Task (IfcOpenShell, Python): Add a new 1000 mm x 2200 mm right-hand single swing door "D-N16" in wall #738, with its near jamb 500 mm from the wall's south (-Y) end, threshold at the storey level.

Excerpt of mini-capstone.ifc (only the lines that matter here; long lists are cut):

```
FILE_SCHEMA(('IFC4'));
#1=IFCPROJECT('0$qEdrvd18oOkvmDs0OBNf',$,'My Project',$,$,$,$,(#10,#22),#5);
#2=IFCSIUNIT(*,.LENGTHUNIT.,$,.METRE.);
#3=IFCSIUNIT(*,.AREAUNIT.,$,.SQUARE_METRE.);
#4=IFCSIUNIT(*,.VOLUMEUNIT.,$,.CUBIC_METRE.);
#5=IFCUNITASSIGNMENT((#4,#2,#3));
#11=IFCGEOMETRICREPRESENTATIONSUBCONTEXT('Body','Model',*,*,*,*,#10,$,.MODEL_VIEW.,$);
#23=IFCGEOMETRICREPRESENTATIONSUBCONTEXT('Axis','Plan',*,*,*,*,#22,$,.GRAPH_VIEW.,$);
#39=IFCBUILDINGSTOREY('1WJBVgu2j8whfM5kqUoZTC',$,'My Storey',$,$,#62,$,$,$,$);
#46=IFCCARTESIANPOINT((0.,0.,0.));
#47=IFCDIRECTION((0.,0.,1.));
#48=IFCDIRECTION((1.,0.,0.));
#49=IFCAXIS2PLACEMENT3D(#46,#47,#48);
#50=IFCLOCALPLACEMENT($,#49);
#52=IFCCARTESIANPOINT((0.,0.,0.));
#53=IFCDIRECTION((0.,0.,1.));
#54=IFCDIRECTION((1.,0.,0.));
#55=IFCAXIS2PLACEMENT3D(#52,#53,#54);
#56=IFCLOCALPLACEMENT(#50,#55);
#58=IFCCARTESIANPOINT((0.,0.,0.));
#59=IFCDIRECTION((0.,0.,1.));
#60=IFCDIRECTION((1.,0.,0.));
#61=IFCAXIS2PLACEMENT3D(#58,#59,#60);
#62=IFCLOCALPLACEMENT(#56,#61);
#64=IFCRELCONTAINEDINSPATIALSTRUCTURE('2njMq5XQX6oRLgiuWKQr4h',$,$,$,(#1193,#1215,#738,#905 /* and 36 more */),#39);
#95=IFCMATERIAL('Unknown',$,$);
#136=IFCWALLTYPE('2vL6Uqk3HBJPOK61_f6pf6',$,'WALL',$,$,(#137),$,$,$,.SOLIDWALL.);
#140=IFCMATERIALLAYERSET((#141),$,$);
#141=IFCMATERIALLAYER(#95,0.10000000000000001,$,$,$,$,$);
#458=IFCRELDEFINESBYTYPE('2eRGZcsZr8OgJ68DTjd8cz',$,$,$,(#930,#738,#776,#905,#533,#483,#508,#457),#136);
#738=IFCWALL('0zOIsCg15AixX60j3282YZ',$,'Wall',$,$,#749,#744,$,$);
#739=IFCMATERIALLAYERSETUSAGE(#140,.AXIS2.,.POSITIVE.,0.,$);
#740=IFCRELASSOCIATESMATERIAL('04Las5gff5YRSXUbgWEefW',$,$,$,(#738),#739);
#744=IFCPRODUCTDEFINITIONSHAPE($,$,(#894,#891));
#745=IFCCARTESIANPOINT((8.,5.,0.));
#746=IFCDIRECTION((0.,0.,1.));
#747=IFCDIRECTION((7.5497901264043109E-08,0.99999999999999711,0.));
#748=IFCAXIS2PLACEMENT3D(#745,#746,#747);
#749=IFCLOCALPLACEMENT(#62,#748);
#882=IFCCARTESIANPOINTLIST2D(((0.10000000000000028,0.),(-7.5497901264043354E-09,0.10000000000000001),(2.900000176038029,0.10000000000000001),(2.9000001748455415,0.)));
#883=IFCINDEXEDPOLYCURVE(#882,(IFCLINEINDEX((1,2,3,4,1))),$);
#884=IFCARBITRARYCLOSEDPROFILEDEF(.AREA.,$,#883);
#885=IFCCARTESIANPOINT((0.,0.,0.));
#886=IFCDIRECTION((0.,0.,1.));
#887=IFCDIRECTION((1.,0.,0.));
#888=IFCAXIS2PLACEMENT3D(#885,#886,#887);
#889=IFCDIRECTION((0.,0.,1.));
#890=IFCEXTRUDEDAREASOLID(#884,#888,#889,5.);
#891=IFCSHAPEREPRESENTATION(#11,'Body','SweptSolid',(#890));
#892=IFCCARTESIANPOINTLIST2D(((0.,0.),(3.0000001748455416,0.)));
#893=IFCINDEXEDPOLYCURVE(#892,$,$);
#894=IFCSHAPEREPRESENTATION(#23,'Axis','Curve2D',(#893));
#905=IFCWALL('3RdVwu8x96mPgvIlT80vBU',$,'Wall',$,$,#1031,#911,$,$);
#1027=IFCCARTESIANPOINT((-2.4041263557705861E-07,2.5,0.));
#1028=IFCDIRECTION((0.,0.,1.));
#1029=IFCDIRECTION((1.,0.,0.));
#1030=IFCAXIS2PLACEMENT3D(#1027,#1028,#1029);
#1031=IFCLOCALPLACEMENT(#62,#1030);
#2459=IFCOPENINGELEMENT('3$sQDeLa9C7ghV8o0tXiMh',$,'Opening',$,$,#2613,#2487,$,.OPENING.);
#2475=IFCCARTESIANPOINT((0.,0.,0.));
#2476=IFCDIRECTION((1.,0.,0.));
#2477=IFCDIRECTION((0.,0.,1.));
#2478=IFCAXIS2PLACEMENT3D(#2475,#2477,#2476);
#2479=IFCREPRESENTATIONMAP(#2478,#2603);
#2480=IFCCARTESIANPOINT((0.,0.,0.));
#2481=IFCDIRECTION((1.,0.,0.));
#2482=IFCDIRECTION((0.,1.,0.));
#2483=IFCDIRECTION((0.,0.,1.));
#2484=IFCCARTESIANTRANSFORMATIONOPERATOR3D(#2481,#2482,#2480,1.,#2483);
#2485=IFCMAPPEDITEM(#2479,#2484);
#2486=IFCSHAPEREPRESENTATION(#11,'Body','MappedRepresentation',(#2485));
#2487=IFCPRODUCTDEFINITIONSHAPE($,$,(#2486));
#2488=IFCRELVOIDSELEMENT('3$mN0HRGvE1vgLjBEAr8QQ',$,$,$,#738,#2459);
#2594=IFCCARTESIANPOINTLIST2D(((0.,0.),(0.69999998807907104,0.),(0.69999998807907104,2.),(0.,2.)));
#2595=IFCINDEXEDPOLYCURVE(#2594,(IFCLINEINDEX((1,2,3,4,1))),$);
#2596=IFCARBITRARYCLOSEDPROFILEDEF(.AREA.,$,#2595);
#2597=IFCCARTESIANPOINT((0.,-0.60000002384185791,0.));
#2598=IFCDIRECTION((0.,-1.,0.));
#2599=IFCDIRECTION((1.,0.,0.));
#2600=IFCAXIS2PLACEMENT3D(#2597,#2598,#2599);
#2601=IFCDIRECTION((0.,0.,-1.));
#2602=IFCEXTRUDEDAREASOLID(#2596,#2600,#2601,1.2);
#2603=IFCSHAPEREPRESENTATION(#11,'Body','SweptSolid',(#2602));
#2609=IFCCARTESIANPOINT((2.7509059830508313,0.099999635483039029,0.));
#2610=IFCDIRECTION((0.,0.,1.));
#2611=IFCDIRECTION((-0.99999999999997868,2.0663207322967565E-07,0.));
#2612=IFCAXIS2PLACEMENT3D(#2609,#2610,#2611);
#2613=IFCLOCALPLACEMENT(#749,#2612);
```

```python
import numpy as np
import ifcopenshell
import ifcopenshell.api.feature
import ifcopenshell.api.geometry
import ifcopenshell.api.root
import ifcopenshell.api.spatial
import ifcopenshell.geom
import ifcopenshell.util.element
import ifcopenshell.util.placement
import ifcopenshell.util.representation
import ifcopenshell.util.shape
import ifcopenshell.util.unit

model = ifcopenshell.open("mini-capstone.ifc")
unit_scale = ifcopenshell.util.unit.calculate_unit_scale(model)
settings = ifcopenshell.geom.settings()


def volume(element):
    """Net volume in cubic metres, openings subtracted."""
    shape = ifcopenshell.geom.create_shape(settings, element)
    return ifcopenshell.util.shape.get_volume(shape.geometry)


wall = model.by_guid("0zOIsCg15AixX60j3282YZ")
storey = ifcopenshell.util.element.get_container(wall, ifc_class="IfcBuildingStorey")
context = ifcopenshell.util.representation.get_context(model, "Model", "Body", "MODEL_VIEW")
before = volume(wall)

width, height, from_end, sill = 1, 2.2, 0.5, 0.0  # metres

# The wall runs along its own X axis, and the end named is its -X end.
wall_shape = ifcopenshell.geom.create_shape(settings, wall)
x, y, z = ifcopenshell.util.shape.get_vertices(wall_shape.geometry).T
start = x.min() + from_end
face, thickness = float(y.min()), float(y.max() - y.min())
wall_matrix = ifcopenshell.util.placement.get_local_placement(wall.ObjectPlacement)
level = ifcopenshell.util.placement.get_local_placement(storey.ObjectPlacement)[2, 3]


def in_wall(x, y):
    """Placement at x, y metres in the wall's axes, at sill height."""
    matrix = wall_matrix.copy()
    matrix[:, 3] = wall_matrix @ np.array([x / unit_scale, y / unit_scale, 0.0, 1.0])
    matrix[2, 3] = level + sill / unit_scale
    return matrix


# Opening: a box that overshoots both wall faces by 50 mm.
opening = ifcopenshell.api.root.create_entity(model, ifc_class="IfcOpeningElement", predefined_type="OPENING")
box = ifcopenshell.api.geometry.add_wall_representation(
    model, context=context, length=width, height=height, thickness=thickness + 0.1
)
ifcopenshell.api.geometry.assign_representation(model, product=opening, representation=box)
ifcopenshell.api.geometry.edit_object_placement(model, product=opening, matrix=in_wall(start, face - 0.05), is_si=False)
ifcopenshell.api.feature.add_feature(model, feature=opening, element=wall)

door = ifcopenshell.api.root.create_entity(model, ifc_class="IfcDoor", name="D-N16", predefined_type="DOOR")
door.OverallWidth, door.OverallHeight = width / unit_scale, height / unit_scale
door.OperationType = "SINGLE_SWING_RIGHT"
body = ifcopenshell.api.geometry.add_door_representation(
    model,
    context=context,
    overall_width=door.OverallWidth,
    overall_height=door.OverallHeight,
    operation_type="SINGLE_SWING_RIGHT",
    lining_properties={"LiningDepth": thickness / unit_scale, "ThresholdDepth": thickness / unit_scale},
)
ifcopenshell.api.geometry.assign_representation(model, product=door, representation=body)
ifcopenshell.api.spatial.assign_container(model, products=[door], relating_structure=storey)
ifcopenshell.api.feature.add_filling(model, opening=opening, element=door)

# The lining spans the wall, so the door starts at the wall face.
ifcopenshell.api.geometry.edit_object_placement(model, product=door, matrix=in_wall(start, face), is_si=False)

after = volume(wall)

print(f"wall volume {before:.3f} -> {after:.3f} m3")

model.write("mini-capstone_updated.ifc")
```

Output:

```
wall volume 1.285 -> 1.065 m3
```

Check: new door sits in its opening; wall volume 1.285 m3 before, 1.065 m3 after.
